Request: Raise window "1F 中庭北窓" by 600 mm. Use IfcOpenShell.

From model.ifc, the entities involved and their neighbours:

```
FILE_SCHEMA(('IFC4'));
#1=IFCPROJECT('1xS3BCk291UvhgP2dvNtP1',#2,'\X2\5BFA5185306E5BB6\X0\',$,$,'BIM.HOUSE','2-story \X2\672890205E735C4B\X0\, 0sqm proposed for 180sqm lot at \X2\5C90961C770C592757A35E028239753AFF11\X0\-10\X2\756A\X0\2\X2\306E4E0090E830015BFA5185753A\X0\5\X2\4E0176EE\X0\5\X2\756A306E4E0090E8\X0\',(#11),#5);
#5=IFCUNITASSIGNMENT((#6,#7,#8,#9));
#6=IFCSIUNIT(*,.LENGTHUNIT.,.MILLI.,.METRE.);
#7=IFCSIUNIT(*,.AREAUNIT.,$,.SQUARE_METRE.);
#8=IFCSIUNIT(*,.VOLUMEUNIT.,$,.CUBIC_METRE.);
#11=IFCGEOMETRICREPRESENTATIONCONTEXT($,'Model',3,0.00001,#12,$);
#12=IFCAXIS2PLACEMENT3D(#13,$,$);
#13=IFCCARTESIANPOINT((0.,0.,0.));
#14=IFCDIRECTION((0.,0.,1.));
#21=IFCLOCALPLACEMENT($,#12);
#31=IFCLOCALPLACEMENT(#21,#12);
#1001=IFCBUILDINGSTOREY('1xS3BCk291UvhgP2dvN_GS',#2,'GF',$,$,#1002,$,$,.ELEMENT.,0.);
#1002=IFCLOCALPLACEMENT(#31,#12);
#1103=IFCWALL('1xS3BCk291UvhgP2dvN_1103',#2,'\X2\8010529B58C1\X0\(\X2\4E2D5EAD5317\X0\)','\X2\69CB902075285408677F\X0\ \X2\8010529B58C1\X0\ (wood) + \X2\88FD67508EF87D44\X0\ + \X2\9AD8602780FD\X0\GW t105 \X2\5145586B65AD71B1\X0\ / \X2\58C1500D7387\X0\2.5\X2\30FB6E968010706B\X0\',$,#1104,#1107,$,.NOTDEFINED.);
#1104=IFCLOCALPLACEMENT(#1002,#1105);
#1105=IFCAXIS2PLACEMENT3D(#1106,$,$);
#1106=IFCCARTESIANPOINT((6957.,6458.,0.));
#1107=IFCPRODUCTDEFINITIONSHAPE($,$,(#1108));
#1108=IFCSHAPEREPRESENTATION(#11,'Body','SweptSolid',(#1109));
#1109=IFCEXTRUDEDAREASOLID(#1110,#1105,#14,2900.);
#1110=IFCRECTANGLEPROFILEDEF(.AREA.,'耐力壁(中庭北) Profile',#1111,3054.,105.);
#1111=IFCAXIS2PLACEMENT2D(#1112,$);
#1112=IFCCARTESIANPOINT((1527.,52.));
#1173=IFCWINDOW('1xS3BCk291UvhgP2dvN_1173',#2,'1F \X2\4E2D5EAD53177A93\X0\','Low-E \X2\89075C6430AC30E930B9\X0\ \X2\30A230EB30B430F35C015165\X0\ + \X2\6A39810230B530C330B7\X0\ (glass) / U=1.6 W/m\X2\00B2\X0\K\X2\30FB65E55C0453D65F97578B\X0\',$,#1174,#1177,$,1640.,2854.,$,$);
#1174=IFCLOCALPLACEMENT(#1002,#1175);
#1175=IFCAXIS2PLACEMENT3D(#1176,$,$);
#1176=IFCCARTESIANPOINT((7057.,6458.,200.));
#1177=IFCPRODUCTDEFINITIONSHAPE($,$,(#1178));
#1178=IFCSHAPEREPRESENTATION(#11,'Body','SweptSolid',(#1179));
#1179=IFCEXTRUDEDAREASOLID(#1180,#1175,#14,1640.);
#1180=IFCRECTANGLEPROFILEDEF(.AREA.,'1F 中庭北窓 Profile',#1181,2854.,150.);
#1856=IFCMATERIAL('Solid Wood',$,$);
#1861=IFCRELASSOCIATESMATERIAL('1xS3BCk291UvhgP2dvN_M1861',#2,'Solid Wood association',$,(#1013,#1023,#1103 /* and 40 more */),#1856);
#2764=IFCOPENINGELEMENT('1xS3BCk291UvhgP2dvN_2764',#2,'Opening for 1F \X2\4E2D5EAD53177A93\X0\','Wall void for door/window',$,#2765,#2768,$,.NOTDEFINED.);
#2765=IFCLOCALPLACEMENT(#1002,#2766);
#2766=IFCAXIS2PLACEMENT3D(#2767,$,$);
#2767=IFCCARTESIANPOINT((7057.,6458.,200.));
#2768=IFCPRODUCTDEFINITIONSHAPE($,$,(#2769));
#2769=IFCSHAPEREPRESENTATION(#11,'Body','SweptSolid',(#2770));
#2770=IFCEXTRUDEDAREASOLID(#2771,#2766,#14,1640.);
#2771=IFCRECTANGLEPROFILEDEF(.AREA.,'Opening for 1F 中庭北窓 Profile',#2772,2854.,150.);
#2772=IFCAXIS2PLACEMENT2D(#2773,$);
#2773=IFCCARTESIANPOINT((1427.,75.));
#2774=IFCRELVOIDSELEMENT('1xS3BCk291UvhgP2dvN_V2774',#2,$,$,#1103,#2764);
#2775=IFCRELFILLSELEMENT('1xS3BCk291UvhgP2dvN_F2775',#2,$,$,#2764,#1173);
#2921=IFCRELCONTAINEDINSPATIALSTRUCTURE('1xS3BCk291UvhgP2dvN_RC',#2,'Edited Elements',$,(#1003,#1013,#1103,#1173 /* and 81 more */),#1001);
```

```python
import numpy as np
import ifcopenshell
import ifcopenshell.api.geometry
import ifcopenshell.util.placement
import ifcopenshell.util.unit

model = ifcopenshell.open("model.ifc")
unit_scale = ifcopenshell.util.unit.calculate_unit_scale(model)

window = model.by_guid("1xS3BCk291UvhgP2dvN_1173")
opening = window.FillsVoids[0].RelatingOpeningElement
dz = 600.0

shift = np.array([0.0, 0.0, dz])
# The window is not placed relative to its opening, so move both.
for product in (opening, window):
    matrix = ifcopenshell.util.placement.get_local_placement(product.ObjectPlacement)
    matrix[:3, 3] += shift
    ifcopenshell.api.geometry.edit_object_placement(model, product=product, matrix=matrix, is_si=False)

print(f"moved by {dz * unit_scale:+.3f} m")

model.write("model_updated.ifc")
```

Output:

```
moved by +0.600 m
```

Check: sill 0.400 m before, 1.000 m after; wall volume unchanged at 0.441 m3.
